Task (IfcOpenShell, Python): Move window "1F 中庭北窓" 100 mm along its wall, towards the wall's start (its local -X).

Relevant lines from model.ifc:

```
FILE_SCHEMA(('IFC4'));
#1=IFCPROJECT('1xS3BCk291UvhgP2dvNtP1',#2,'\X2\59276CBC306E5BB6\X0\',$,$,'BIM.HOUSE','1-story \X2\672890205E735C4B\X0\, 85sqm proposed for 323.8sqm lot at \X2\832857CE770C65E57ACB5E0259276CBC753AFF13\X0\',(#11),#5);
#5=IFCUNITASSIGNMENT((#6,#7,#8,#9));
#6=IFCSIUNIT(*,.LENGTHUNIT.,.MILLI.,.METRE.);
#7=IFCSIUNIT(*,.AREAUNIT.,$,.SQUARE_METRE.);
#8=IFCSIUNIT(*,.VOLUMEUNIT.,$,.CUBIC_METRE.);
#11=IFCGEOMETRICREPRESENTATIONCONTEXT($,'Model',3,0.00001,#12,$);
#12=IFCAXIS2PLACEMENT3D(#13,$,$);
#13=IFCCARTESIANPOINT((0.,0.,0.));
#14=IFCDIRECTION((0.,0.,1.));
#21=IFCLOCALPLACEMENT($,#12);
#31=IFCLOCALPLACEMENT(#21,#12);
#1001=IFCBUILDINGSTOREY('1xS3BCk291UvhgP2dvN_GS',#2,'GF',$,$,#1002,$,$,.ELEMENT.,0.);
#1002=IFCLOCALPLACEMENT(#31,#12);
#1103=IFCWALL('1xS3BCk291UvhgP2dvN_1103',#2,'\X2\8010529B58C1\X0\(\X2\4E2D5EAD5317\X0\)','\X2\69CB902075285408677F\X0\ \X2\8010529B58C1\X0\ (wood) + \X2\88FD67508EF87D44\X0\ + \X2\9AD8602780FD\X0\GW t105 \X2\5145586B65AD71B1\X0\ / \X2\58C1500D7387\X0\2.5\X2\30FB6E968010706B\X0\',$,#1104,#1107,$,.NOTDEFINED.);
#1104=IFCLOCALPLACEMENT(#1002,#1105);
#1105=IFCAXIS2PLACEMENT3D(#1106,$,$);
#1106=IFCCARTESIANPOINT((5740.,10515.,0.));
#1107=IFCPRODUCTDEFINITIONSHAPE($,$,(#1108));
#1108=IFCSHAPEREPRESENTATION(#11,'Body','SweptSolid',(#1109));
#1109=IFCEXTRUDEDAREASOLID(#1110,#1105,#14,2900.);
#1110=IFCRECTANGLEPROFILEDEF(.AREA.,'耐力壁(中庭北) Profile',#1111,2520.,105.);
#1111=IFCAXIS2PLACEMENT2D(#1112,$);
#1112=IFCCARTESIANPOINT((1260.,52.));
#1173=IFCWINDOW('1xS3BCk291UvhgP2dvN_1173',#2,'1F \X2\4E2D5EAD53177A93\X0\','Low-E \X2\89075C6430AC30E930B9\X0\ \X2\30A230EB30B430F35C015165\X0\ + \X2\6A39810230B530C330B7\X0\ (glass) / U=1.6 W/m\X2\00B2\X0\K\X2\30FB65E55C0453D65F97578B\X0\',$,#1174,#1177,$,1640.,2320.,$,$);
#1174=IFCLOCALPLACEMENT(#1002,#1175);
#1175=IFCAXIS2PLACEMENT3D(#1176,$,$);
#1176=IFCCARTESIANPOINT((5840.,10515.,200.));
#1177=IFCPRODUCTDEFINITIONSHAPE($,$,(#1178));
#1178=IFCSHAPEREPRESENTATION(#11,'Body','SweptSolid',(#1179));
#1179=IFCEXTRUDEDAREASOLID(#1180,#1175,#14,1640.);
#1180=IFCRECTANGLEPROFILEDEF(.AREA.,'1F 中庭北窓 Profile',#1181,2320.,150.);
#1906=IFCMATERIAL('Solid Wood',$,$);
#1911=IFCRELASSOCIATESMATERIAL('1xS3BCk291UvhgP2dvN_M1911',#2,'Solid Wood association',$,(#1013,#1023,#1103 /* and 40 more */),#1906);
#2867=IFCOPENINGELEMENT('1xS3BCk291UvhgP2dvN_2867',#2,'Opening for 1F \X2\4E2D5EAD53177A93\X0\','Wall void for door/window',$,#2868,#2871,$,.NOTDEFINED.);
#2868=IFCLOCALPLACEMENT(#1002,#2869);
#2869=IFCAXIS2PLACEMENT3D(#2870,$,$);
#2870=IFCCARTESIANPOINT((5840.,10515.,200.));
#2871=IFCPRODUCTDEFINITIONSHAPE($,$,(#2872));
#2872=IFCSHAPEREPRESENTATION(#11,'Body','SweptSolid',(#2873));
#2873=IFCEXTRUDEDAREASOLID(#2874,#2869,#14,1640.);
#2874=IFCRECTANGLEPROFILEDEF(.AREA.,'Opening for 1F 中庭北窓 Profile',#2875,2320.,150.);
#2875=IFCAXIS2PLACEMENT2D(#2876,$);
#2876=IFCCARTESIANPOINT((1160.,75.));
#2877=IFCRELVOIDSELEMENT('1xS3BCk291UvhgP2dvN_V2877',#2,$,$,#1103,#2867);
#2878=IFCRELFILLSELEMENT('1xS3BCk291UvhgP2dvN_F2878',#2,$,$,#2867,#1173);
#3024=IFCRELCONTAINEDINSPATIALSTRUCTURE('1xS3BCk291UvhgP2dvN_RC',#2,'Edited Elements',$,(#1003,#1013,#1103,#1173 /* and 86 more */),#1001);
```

```python
import ifcopenshell
import ifcopenshell.api.geometry
import ifcopenshell.util.placement
import ifcopenshell.util.unit

model = ifcopenshell.open("model.ifc")
unit_scale = ifcopenshell.util.unit.calculate_unit_scale(model)

window = model.by_guid("1xS3BCk291UvhgP2dvN_1173")
opening = window.FillsVoids[0].RelatingOpeningElement
wall = opening.VoidsElements[0].RelatingBuildingElement

wall_matrix = ifcopenshell.util.placement.get_local_placement(wall.ObjectPlacement)
shift = wall_matrix[:3, 0] * -0.1 / unit_scale
before = ifcopenshell.util.placement.get_local_placement(window.ObjectPlacement)[:3, 3].copy()

# The window is not placed relative to its opening, so move both.
for product in (opening, window):
    matrix = ifcopenshell.util.placement.get_local_placement(product.ObjectPlacement)
    matrix[:3, 3] += shift
    ifcopenshell.api.geometry.edit_object_placement(model, product=product, matrix=matrix, is_si=False)

after = ifcopenshell.util.placement.get_local_placement(window.ObjectPlacement)[:3, 3]
print("window moved by", (after - before).round(3) + 0.0)

model.write("model_rev.ifc")
```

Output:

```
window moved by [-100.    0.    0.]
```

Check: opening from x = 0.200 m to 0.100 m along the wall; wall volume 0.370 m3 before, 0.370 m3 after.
